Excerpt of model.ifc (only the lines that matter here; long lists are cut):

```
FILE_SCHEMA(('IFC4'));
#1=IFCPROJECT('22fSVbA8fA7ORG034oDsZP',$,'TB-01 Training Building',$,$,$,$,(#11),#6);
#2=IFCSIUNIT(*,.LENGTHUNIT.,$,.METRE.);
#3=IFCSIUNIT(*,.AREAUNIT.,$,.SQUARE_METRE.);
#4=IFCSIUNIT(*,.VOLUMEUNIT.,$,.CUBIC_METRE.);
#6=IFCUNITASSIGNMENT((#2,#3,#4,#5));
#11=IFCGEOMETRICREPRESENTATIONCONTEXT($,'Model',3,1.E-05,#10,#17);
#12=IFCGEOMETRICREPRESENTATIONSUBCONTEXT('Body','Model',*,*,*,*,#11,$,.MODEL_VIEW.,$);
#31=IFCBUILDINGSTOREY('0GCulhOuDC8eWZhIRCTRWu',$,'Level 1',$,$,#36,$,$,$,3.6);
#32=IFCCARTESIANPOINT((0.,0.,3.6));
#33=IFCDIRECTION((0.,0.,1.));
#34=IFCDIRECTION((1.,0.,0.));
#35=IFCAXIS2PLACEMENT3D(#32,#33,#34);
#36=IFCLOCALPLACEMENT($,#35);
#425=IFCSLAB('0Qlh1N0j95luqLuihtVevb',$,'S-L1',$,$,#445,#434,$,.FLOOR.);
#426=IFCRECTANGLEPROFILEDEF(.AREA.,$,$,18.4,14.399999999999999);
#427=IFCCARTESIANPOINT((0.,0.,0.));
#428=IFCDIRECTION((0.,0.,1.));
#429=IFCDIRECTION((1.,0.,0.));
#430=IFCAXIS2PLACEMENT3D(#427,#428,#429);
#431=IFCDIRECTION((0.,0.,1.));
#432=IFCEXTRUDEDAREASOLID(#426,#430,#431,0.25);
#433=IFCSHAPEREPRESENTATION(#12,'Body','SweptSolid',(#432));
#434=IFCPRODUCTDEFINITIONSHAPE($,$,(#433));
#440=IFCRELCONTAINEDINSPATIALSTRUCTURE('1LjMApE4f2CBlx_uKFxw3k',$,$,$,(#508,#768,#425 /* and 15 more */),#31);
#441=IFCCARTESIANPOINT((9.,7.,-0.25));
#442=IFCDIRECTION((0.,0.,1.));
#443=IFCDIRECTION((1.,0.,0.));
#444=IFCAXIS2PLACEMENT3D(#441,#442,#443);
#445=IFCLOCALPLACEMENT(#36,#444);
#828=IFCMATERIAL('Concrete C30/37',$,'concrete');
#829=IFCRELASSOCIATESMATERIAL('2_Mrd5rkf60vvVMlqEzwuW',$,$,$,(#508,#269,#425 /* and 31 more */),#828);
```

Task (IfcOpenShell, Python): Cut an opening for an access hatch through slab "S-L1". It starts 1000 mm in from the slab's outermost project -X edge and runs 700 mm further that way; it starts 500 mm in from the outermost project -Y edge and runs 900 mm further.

```python
import numpy as np
import ifcopenshell
import ifcopenshell.api.feature
import ifcopenshell.api.geometry
import ifcopenshell.api.root
import ifcopenshell.geom
import ifcopenshell.util.placement
import ifcopenshell.util.representation
import ifcopenshell.util.shape
import ifcopenshell.util.unit

model = ifcopenshell.open("model.ifc")
unit_scale = ifcopenshell.util.unit.calculate_unit_scale(model)
settings = ifcopenshell.geom.settings()


def volume(element):
    """Net volume in cubic metres, openings subtracted."""
    shape = ifcopenshell.geom.create_shape(settings, element)
    return ifcopenshell.util.shape.get_volume(shape.geometry)


slab = model.by_guid("0Qlh1N0j95luqLuihtVevb")
before = volume(slab)

# Extent in the slab's own axes, in metres. The edges named are its -X and -Y sides.
slab_shape = ifcopenshell.geom.create_shape(settings, slab)
vertices = ifcopenshell.util.shape.get_vertices(slab_shape.geometry)
x_min, y_min, bottom = vertices.min(axis=0)
top = vertices[:, 2].max()

opening = ifcopenshell.api.root.create_entity(model, ifc_class="IfcOpeningElement", name="Access hatch opening", predefined_type="OPENING")
context = ifcopenshell.util.representation.get_context(model, "Model", "Body", "MODEL_VIEW")
width, depth = 0.7, 0.9
outline = [(0.0, 0.0), (width, 0.0), (width, depth), (0.0, depth), (0.0, 0.0)]
# Overshoot both faces by 50 mm so the cut is clean.
shape = ifcopenshell.api.geometry.add_slab_representation(
    model, context=context, depth=top - bottom + 0.1, polyline=outline
)
ifcopenshell.api.geometry.assign_representation(model, product=opening, representation=shape)

matrix = ifcopenshell.util.placement.get_local_placement(slab.ObjectPlacement)
matrix[:, 3] = matrix @ np.append(np.array([x_min + 1, y_min + 0.5, bottom - 0.05]) / unit_scale, 1.0)
ifcopenshell.api.geometry.edit_object_placement(model, product=opening, matrix=matrix, is_si=False)
ifcopenshell.api.feature.add_feature(model, feature=opening, element=slab)

after = volume(slab)

print(f"slab volume {before:.3f} -> {after:.3f} m3")

model.write("model_edited.ifc")
```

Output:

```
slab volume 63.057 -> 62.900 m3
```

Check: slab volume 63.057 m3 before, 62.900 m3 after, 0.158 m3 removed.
